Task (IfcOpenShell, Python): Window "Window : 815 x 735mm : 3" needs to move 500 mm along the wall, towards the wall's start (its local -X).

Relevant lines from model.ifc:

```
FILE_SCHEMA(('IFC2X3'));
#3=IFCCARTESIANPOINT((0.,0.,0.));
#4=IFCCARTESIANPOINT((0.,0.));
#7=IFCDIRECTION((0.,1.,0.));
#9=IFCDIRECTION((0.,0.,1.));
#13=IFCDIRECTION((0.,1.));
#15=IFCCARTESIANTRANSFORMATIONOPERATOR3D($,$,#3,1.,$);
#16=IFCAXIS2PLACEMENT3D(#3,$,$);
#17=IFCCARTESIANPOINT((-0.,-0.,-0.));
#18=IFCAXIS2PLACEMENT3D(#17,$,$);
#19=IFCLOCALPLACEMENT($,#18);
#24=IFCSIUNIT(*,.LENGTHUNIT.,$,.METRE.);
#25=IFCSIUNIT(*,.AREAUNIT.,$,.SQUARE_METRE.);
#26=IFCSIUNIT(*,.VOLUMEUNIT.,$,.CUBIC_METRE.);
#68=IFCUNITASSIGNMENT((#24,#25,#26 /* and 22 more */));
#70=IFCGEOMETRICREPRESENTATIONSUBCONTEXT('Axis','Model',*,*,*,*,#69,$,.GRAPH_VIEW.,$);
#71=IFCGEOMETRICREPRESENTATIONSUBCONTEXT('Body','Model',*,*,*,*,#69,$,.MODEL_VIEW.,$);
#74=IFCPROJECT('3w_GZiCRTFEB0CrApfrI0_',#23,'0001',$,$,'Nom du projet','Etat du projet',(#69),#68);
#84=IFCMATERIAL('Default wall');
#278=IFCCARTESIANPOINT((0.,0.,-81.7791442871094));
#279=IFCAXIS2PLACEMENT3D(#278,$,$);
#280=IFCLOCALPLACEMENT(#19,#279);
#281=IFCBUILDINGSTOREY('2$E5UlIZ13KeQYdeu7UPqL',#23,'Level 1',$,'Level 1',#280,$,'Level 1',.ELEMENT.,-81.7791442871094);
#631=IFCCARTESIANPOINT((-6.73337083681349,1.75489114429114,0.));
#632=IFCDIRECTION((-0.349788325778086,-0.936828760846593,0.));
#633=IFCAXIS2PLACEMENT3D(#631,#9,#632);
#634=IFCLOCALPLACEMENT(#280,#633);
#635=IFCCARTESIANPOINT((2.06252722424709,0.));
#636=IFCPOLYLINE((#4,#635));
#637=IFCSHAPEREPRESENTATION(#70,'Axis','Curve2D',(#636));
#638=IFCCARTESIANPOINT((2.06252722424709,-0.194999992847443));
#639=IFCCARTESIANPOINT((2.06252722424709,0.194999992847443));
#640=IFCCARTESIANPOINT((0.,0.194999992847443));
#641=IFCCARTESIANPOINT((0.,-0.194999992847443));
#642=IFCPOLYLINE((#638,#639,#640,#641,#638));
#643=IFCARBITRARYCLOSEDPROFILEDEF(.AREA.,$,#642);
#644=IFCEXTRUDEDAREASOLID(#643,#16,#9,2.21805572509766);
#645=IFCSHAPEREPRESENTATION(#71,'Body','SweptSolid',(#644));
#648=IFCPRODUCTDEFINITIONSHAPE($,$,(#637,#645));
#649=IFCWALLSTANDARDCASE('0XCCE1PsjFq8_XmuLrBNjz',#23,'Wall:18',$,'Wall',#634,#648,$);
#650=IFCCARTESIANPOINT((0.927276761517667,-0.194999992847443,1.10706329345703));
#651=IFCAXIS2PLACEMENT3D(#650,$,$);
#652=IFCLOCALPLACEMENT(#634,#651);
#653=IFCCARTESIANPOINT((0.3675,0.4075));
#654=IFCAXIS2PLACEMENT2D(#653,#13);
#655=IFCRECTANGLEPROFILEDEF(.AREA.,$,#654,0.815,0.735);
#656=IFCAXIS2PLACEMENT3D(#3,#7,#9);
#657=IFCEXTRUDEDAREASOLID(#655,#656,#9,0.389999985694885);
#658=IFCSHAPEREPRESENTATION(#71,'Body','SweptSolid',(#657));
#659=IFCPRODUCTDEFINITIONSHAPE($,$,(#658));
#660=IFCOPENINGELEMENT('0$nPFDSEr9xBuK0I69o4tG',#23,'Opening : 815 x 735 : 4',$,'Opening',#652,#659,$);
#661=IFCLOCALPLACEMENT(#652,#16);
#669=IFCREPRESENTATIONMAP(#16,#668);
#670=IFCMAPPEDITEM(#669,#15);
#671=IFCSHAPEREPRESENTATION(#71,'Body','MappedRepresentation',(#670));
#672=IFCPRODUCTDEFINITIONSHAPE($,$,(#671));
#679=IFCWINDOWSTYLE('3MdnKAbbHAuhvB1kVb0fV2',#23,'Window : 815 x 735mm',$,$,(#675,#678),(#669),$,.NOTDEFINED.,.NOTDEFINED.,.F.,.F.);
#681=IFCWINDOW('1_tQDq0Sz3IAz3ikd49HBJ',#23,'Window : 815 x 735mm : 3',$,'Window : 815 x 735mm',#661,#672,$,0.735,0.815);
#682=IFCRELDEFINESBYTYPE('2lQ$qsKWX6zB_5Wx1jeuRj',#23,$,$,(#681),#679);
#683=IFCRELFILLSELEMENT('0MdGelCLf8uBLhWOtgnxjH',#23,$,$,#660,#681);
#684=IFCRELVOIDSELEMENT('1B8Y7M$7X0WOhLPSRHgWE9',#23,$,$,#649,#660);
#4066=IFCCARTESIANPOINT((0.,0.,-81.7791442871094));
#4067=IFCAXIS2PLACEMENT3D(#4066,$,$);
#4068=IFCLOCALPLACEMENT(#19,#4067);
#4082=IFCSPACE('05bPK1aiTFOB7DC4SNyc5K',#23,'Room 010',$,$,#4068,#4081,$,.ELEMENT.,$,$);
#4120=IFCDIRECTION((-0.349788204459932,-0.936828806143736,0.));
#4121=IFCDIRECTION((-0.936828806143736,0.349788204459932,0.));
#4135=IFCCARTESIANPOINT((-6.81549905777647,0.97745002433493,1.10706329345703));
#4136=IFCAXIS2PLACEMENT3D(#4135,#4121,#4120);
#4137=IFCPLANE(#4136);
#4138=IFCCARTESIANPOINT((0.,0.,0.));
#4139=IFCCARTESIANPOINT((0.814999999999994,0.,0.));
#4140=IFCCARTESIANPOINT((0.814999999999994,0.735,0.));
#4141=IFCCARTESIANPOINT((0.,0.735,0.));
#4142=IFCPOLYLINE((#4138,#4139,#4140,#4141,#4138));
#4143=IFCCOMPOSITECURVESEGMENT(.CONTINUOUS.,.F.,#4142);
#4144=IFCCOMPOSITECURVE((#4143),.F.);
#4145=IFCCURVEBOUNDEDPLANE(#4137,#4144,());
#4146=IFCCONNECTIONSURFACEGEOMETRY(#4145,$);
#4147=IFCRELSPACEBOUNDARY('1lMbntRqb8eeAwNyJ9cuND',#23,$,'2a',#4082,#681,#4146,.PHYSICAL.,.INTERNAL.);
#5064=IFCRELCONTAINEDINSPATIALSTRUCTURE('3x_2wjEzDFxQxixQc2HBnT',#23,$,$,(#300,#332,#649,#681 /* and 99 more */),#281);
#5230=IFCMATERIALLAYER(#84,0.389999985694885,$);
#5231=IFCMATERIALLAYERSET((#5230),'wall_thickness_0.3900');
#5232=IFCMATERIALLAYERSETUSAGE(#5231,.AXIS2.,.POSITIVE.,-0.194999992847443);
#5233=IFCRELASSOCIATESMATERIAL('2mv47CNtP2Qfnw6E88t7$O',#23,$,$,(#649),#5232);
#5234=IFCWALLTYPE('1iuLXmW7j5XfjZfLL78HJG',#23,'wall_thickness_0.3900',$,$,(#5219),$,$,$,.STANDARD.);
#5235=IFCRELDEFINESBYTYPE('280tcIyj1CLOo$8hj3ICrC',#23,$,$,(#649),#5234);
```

```python
import numpy as np
import ifcopenshell
import ifcopenshell.api.geometry
import ifcopenshell.util.placement
import ifcopenshell.util.unit

model = ifcopenshell.open("model.ifc")
unit_scale = ifcopenshell.util.unit.calculate_unit_scale(model)

window = model.by_guid("1_tQDq0Sz3IAz3ikd49HBJ")
opening = window.FillsVoids[0].RelatingOpeningElement
wall = opening.VoidsElements[0].RelatingBuildingElement

wall_matrix = ifcopenshell.util.placement.get_local_placement(wall.ObjectPlacement)
shift = wall_matrix[:3, 0] * -0.5 / unit_scale
before = ifcopenshell.util.placement.get_local_placement(window.ObjectPlacement)[:3, 3].copy()

# The window is placed relative to its opening, so it follows when the opening moves.
matrix = ifcopenshell.util.placement.get_local_placement(opening.ObjectPlacement)
matrix[:3, 3] += shift
ifcopenshell.api.geometry.edit_object_placement(
    model, product=opening, matrix=matrix, is_si=False, should_transform_children=True
)

# Space boundary surfaces are stored in each space's coordinates; move them too.
for rel in window.ProvidesBoundaries:
    if not rel.ConnectionGeometry:
        continue
    surface = rel.ConnectionGeometry.SurfaceOnRelatingElement.BasisSurface
    space_matrix = ifcopenshell.util.placement.get_local_placement(rel.RelatingSpace.ObjectPlacement)
    point = np.array(surface.Position.Location.Coordinates) + space_matrix[:3, :3].T @ shift
    surface.Position = model.createIfcAxis2Placement3D(
        model.createIfcCartesianPoint(point.tolist()), surface.Position.Axis, surface.Position.RefDirection
    )

after = ifcopenshell.util.placement.get_local_placement(window.ObjectPlacement)[:3, 3]
print("window moved by", (after - before).round(3) + 0.0)

model.write("model_updated.ifc")
```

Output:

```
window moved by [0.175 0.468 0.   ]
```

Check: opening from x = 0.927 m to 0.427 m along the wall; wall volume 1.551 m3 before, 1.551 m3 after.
